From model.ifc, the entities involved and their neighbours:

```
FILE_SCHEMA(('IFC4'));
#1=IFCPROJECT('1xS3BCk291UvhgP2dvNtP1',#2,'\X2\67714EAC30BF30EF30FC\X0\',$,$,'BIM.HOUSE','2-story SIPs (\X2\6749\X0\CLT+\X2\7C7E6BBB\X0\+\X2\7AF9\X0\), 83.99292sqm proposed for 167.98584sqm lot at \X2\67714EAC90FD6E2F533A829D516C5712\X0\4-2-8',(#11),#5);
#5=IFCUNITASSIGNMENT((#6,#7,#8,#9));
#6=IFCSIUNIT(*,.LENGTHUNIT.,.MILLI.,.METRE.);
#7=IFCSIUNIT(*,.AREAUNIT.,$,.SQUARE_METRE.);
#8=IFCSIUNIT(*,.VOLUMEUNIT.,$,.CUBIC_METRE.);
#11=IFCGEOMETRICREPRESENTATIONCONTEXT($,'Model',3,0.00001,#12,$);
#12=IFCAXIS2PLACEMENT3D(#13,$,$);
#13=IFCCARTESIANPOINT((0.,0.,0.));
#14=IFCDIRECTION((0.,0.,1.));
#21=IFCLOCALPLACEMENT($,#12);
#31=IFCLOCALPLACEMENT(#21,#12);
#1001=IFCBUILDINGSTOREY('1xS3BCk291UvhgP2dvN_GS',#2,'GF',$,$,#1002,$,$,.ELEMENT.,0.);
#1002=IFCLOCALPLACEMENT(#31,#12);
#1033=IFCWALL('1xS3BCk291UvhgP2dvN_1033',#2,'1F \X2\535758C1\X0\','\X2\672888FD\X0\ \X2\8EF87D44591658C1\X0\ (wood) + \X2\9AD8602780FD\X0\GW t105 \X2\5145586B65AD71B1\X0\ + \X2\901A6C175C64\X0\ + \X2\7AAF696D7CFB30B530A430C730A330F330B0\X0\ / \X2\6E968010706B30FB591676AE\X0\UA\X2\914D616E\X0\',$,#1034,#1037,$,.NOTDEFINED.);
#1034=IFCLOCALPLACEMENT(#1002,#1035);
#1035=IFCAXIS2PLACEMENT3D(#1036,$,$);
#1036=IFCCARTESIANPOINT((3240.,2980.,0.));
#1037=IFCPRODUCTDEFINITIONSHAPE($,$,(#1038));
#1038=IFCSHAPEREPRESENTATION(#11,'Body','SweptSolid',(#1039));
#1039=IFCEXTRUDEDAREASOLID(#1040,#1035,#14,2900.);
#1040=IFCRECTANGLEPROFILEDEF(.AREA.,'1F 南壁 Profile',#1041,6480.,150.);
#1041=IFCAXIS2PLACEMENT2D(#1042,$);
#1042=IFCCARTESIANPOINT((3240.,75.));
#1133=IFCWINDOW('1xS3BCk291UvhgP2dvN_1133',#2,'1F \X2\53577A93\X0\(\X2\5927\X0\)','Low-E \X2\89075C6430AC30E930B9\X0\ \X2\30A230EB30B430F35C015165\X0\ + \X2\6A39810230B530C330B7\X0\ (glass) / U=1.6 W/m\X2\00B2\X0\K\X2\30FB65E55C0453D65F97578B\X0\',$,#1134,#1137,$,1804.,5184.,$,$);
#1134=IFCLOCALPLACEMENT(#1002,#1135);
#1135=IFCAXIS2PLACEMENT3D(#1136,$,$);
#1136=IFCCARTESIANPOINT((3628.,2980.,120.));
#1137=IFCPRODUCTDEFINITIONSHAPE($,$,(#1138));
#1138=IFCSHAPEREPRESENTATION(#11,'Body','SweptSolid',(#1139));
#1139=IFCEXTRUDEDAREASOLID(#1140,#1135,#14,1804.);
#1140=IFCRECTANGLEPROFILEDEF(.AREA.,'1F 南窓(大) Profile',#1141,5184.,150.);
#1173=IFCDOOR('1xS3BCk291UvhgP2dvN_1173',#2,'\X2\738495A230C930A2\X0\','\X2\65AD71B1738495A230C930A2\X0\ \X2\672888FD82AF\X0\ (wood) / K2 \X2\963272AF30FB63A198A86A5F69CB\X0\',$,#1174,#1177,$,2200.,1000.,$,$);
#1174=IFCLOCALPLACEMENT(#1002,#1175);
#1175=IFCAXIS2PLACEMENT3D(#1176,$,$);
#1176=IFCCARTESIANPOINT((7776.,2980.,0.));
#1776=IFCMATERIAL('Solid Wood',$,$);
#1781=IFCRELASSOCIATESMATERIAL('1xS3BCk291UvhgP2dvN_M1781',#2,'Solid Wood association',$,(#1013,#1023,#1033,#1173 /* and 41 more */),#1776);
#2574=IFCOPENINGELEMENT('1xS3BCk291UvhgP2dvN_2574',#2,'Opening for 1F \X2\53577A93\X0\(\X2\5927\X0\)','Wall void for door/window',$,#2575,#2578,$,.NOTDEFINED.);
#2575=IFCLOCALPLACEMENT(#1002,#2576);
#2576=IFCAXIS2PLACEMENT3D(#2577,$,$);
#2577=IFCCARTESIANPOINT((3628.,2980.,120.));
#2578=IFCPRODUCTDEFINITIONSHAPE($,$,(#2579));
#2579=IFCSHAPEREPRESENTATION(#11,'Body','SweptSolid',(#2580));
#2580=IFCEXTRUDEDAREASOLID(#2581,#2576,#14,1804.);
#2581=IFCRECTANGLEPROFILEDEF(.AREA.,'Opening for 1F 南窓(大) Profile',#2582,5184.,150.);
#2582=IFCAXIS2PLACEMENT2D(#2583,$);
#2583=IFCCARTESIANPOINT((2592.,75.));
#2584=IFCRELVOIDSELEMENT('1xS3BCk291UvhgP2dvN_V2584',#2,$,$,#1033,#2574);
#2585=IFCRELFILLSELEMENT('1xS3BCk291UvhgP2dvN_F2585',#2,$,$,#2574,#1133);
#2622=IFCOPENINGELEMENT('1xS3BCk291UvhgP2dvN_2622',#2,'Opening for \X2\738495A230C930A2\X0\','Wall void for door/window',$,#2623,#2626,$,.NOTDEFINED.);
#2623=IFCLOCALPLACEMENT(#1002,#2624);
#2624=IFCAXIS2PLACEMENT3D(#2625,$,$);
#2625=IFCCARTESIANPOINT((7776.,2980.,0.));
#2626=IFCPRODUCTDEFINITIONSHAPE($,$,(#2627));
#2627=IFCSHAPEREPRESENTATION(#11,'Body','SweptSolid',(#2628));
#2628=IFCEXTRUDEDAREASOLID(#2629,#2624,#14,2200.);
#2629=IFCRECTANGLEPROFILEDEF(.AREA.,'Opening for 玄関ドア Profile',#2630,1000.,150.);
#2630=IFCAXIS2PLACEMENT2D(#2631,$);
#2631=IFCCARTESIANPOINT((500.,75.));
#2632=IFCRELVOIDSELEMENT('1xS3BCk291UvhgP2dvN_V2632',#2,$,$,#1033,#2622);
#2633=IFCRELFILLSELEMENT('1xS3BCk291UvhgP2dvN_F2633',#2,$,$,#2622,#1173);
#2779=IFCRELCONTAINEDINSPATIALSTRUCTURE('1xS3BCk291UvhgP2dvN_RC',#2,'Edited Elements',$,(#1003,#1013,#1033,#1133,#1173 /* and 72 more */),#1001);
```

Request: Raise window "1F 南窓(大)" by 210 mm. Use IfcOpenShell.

```python
import numpy as np
import ifcopenshell
import ifcopenshell.api.geometry
import ifcopenshell.util.placement
import ifcopenshell.util.unit

model = ifcopenshell.open("model.ifc")
unit_scale = ifcopenshell.util.unit.calculate_unit_scale(model)

window = model.by_guid("1xS3BCk291UvhgP2dvN_1133")
opening = window.FillsVoids[0].RelatingOpeningElement
dz = 210.0

shift = np.array([0.0, 0.0, dz])
# The window is not placed relative to its opening, so move both.
for product in (opening, window):
    matrix = ifcopenshell.util.placement.get_local_placement(product.ObjectPlacement)
    matrix[:3, 3] += shift
    ifcopenshell.api.geometry.edit_object_placement(model, product=product, matrix=matrix, is_si=False)

print(f"moved by {dz * unit_scale:+.3f} m")

model.write("model_edited.ifc")
```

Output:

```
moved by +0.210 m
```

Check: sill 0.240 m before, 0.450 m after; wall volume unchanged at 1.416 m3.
